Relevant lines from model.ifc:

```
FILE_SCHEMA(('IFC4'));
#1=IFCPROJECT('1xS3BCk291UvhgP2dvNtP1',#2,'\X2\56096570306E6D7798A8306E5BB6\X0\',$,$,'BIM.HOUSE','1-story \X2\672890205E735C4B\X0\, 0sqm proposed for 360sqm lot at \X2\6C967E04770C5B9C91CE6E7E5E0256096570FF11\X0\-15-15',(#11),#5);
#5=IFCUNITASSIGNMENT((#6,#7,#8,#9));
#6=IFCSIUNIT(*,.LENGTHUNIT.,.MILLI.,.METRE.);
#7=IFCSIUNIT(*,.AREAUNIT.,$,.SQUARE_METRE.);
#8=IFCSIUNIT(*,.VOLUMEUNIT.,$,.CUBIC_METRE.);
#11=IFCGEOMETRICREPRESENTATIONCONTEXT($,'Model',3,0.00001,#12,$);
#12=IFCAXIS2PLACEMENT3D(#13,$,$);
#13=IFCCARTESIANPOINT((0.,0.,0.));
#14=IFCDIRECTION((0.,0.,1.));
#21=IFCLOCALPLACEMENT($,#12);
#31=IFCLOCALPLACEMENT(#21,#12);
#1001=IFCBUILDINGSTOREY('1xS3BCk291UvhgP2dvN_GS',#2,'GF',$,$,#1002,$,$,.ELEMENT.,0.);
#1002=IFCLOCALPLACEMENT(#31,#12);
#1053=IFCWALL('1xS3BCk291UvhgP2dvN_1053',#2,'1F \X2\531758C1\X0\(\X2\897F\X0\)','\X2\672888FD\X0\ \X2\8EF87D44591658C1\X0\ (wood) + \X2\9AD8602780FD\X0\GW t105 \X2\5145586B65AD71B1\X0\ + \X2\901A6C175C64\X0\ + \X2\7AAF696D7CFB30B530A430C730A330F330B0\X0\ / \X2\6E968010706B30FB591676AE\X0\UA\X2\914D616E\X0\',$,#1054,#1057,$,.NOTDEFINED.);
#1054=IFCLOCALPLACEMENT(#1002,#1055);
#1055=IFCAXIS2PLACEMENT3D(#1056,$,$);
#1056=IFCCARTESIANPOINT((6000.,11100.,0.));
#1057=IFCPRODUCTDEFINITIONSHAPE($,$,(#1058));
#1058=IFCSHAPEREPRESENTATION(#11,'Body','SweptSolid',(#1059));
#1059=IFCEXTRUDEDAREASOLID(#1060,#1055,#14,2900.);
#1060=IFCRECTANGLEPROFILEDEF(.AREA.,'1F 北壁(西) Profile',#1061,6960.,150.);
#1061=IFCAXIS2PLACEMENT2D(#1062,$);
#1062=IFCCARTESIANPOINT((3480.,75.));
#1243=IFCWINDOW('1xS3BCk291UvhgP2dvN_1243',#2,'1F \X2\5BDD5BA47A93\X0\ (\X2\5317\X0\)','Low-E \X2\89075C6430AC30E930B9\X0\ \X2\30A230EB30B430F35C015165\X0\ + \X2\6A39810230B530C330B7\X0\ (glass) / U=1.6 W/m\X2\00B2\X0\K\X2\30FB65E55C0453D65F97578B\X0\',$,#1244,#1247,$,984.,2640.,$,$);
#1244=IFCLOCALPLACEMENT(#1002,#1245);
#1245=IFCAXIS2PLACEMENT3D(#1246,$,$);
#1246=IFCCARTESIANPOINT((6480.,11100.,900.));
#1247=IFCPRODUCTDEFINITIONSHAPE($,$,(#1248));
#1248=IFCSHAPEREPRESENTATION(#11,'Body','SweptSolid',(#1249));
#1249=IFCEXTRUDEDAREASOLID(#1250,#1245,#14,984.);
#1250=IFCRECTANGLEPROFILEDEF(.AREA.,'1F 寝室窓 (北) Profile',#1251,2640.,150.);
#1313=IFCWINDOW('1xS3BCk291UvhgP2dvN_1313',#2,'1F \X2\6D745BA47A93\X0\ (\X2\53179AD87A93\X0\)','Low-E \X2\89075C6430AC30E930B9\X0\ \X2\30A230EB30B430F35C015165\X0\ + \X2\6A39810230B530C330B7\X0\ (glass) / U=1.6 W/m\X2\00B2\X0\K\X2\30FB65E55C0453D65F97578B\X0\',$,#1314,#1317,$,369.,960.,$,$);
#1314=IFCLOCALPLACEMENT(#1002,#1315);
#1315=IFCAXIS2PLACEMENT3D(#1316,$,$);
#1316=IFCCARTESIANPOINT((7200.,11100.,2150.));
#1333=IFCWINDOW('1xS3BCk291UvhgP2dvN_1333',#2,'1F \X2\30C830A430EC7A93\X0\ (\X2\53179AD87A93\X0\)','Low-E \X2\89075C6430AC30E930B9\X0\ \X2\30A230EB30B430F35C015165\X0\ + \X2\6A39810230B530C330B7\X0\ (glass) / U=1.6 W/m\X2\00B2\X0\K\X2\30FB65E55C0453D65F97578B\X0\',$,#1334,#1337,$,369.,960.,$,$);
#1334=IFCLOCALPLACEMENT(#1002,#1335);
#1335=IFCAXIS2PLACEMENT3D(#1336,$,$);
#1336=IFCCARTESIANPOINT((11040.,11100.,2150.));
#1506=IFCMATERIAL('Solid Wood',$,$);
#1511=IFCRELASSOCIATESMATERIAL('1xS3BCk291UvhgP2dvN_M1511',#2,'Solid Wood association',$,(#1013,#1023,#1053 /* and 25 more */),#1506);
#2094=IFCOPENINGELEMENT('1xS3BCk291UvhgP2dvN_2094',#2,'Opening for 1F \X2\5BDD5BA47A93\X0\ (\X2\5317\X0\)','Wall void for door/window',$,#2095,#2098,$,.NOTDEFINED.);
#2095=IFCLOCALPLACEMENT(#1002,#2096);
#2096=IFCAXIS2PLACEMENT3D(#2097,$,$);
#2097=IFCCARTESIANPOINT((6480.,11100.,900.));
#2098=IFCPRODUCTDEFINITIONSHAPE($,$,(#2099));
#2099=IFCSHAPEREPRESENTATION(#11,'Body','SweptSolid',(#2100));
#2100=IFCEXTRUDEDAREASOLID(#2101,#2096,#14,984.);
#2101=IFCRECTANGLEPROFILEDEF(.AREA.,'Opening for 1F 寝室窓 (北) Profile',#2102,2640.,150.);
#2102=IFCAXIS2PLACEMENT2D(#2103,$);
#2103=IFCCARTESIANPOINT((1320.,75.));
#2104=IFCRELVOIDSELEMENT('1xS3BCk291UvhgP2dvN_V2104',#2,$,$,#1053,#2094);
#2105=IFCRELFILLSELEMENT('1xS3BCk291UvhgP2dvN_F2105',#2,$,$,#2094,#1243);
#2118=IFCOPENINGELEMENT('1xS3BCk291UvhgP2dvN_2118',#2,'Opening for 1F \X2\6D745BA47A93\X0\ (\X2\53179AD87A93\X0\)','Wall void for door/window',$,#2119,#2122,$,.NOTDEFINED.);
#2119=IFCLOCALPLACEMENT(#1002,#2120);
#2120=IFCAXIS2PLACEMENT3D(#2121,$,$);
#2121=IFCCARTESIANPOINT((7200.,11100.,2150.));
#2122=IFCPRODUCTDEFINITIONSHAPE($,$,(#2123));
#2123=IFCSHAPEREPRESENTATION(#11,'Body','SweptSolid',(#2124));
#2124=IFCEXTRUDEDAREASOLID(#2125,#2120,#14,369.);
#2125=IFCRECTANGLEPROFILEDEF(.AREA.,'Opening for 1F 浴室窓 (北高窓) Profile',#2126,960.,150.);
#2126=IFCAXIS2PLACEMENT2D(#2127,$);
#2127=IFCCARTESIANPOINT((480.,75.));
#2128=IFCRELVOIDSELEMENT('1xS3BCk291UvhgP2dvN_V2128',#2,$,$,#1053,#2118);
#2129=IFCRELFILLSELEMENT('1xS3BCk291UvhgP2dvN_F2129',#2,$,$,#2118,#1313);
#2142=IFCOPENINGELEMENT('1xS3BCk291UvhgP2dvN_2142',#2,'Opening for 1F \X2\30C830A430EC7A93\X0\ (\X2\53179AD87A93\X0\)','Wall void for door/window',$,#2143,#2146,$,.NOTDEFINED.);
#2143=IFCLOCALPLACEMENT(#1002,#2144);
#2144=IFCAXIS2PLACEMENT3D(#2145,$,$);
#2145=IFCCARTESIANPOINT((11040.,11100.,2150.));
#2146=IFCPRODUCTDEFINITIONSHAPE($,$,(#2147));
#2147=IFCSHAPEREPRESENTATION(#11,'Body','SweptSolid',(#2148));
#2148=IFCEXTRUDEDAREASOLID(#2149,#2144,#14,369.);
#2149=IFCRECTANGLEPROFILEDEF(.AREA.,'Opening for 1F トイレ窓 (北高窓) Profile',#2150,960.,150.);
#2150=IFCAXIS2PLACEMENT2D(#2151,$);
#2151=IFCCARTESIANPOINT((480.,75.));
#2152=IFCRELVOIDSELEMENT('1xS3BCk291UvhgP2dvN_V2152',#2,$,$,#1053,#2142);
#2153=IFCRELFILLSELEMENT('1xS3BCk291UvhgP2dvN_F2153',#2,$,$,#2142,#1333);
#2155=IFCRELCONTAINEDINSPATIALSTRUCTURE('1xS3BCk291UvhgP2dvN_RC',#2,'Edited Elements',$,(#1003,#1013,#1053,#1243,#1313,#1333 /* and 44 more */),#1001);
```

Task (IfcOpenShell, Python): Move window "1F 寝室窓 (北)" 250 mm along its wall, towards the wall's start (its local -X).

```python
import ifcopenshell
import ifcopenshell.api.geometry
import ifcopenshell.util.placement

model = ifcopenshell.open("model.ifc")

window = model.by_guid("1xS3BCk291UvhgP2dvN_1243")
opening = window.FillsVoids[0].RelatingOpeningElement
wall = opening.VoidsElements[0].RelatingBuildingElement

wall_matrix = ifcopenshell.util.placement.get_local_placement(wall.ObjectPlacement)
shift = wall_matrix[:3, 0] * -250.0
before = ifcopenshell.util.placement.get_local_placement(window.ObjectPlacement)[:3, 3].copy()

# The window is not placed relative to its opening, so move both.
for product in (opening, window):
    matrix = ifcopenshell.util.placement.get_local_placement(product.ObjectPlacement)
    matrix[:3, 3] += shift
    ifcopenshell.api.geometry.edit_object_placement(model, product=product, matrix=matrix, is_si=False)

after = ifcopenshell.util.placement.get_local_placement(window.ObjectPlacement)[:3, 3]
print("window moved by", (after - before).round(3) + 0.0)

model.write("model_rev.ifc")
```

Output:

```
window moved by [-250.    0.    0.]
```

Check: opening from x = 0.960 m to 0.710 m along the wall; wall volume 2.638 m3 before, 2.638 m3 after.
